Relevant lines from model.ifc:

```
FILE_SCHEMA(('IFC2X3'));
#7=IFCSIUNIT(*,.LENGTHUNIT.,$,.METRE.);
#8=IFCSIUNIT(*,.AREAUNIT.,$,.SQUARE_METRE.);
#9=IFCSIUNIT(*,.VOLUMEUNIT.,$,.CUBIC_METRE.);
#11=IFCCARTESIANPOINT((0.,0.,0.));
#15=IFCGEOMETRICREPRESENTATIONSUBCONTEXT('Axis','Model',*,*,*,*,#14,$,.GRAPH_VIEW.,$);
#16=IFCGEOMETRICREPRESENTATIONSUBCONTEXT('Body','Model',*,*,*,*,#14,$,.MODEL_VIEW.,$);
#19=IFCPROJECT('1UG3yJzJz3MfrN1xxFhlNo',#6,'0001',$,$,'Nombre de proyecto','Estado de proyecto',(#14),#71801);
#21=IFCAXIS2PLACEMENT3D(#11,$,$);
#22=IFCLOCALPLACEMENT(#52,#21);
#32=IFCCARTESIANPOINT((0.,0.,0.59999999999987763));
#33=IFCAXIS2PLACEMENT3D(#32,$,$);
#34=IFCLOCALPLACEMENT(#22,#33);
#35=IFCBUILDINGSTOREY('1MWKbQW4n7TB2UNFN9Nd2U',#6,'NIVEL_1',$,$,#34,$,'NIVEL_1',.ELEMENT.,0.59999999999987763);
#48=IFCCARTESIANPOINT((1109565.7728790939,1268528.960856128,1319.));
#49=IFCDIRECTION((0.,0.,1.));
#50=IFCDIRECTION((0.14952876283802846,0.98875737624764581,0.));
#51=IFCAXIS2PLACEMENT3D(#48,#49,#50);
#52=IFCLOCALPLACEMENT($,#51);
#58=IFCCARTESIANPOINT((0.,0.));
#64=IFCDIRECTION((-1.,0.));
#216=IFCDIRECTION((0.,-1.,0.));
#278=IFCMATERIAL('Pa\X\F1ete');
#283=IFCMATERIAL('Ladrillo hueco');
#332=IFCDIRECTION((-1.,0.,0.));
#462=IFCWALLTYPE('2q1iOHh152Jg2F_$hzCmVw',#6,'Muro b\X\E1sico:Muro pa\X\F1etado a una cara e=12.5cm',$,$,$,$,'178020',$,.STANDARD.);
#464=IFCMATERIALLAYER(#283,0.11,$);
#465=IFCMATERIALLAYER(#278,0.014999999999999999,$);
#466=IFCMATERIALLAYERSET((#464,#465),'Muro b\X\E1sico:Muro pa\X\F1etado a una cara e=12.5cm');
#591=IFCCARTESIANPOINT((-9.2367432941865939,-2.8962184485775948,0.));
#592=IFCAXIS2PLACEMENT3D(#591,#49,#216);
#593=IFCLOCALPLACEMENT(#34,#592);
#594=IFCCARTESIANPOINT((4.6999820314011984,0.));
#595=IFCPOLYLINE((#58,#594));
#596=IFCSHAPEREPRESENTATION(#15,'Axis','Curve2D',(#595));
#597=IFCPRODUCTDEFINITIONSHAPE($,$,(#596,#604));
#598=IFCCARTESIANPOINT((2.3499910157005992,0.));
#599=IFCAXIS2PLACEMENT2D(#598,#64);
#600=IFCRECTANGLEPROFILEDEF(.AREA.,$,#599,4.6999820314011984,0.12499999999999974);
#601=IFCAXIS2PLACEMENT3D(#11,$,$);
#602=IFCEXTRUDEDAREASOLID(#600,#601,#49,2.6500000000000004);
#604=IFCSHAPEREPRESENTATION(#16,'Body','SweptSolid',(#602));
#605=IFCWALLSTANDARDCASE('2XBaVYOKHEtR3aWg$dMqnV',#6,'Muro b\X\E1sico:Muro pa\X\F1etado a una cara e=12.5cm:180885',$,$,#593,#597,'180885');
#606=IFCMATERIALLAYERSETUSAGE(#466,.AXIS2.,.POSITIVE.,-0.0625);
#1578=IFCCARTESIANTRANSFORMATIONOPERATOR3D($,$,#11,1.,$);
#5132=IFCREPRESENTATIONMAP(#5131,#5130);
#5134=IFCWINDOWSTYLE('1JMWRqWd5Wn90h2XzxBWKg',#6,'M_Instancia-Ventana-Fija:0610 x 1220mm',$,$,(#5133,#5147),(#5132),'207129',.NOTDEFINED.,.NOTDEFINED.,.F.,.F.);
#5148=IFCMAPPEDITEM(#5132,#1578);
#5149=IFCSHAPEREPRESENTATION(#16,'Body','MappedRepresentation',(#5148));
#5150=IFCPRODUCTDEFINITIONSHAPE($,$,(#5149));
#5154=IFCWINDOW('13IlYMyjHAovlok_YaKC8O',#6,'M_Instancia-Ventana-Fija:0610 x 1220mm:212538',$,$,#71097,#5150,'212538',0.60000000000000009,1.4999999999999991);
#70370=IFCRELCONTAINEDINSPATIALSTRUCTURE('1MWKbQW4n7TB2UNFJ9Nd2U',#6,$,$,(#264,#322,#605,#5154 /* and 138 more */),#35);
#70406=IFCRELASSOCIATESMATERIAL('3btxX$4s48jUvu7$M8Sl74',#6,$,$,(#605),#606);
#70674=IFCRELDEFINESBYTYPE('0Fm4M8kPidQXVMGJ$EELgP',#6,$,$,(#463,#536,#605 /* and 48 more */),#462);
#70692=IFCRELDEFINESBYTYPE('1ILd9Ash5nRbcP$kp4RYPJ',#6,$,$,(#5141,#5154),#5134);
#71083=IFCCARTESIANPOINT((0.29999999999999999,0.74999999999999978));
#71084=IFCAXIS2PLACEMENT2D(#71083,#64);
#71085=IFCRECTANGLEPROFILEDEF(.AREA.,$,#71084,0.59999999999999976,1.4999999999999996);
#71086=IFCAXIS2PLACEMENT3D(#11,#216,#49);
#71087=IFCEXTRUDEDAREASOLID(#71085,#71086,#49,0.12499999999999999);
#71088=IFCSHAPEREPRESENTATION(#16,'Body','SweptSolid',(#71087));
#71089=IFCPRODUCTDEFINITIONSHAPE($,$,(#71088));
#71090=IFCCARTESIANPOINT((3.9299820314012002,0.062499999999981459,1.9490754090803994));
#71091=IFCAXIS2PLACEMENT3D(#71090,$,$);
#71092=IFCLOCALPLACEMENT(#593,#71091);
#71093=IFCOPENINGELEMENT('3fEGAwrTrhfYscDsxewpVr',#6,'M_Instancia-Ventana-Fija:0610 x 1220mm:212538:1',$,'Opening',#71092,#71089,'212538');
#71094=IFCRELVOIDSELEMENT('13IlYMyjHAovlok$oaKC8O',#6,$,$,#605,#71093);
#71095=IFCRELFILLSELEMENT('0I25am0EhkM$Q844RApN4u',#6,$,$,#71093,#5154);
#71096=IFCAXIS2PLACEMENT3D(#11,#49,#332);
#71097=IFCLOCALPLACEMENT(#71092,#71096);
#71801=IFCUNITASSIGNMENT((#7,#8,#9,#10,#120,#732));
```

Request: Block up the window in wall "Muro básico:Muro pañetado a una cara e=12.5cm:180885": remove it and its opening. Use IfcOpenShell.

```python
import ifcopenshell
import ifcopenshell.api.feature
import ifcopenshell.api.root
import ifcopenshell.geom
import ifcopenshell.util.shape

model = ifcopenshell.open("model.ifc")
settings = ifcopenshell.geom.settings()


def volume(element):
    """Net volume in cubic metres, openings subtracted."""
    shape = ifcopenshell.geom.create_shape(settings, element)
    return ifcopenshell.util.shape.get_volume(shape.geometry)


window = model.by_id(5154)
opening = window.FillsVoids[0].RelatingOpeningElement
wall = opening.VoidsElements[0].RelatingBuildingElement
before = volume(wall)

ifcopenshell.api.root.remove_product(model, product=window)
ifcopenshell.api.feature.remove_feature(model, feature=opening)

after = volume(wall)

print(f"wall volume {before:.3f} -> {after:.3f} m3")

model.write("model_rev.ifc")
```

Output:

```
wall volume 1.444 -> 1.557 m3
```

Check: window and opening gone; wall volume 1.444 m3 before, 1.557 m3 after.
